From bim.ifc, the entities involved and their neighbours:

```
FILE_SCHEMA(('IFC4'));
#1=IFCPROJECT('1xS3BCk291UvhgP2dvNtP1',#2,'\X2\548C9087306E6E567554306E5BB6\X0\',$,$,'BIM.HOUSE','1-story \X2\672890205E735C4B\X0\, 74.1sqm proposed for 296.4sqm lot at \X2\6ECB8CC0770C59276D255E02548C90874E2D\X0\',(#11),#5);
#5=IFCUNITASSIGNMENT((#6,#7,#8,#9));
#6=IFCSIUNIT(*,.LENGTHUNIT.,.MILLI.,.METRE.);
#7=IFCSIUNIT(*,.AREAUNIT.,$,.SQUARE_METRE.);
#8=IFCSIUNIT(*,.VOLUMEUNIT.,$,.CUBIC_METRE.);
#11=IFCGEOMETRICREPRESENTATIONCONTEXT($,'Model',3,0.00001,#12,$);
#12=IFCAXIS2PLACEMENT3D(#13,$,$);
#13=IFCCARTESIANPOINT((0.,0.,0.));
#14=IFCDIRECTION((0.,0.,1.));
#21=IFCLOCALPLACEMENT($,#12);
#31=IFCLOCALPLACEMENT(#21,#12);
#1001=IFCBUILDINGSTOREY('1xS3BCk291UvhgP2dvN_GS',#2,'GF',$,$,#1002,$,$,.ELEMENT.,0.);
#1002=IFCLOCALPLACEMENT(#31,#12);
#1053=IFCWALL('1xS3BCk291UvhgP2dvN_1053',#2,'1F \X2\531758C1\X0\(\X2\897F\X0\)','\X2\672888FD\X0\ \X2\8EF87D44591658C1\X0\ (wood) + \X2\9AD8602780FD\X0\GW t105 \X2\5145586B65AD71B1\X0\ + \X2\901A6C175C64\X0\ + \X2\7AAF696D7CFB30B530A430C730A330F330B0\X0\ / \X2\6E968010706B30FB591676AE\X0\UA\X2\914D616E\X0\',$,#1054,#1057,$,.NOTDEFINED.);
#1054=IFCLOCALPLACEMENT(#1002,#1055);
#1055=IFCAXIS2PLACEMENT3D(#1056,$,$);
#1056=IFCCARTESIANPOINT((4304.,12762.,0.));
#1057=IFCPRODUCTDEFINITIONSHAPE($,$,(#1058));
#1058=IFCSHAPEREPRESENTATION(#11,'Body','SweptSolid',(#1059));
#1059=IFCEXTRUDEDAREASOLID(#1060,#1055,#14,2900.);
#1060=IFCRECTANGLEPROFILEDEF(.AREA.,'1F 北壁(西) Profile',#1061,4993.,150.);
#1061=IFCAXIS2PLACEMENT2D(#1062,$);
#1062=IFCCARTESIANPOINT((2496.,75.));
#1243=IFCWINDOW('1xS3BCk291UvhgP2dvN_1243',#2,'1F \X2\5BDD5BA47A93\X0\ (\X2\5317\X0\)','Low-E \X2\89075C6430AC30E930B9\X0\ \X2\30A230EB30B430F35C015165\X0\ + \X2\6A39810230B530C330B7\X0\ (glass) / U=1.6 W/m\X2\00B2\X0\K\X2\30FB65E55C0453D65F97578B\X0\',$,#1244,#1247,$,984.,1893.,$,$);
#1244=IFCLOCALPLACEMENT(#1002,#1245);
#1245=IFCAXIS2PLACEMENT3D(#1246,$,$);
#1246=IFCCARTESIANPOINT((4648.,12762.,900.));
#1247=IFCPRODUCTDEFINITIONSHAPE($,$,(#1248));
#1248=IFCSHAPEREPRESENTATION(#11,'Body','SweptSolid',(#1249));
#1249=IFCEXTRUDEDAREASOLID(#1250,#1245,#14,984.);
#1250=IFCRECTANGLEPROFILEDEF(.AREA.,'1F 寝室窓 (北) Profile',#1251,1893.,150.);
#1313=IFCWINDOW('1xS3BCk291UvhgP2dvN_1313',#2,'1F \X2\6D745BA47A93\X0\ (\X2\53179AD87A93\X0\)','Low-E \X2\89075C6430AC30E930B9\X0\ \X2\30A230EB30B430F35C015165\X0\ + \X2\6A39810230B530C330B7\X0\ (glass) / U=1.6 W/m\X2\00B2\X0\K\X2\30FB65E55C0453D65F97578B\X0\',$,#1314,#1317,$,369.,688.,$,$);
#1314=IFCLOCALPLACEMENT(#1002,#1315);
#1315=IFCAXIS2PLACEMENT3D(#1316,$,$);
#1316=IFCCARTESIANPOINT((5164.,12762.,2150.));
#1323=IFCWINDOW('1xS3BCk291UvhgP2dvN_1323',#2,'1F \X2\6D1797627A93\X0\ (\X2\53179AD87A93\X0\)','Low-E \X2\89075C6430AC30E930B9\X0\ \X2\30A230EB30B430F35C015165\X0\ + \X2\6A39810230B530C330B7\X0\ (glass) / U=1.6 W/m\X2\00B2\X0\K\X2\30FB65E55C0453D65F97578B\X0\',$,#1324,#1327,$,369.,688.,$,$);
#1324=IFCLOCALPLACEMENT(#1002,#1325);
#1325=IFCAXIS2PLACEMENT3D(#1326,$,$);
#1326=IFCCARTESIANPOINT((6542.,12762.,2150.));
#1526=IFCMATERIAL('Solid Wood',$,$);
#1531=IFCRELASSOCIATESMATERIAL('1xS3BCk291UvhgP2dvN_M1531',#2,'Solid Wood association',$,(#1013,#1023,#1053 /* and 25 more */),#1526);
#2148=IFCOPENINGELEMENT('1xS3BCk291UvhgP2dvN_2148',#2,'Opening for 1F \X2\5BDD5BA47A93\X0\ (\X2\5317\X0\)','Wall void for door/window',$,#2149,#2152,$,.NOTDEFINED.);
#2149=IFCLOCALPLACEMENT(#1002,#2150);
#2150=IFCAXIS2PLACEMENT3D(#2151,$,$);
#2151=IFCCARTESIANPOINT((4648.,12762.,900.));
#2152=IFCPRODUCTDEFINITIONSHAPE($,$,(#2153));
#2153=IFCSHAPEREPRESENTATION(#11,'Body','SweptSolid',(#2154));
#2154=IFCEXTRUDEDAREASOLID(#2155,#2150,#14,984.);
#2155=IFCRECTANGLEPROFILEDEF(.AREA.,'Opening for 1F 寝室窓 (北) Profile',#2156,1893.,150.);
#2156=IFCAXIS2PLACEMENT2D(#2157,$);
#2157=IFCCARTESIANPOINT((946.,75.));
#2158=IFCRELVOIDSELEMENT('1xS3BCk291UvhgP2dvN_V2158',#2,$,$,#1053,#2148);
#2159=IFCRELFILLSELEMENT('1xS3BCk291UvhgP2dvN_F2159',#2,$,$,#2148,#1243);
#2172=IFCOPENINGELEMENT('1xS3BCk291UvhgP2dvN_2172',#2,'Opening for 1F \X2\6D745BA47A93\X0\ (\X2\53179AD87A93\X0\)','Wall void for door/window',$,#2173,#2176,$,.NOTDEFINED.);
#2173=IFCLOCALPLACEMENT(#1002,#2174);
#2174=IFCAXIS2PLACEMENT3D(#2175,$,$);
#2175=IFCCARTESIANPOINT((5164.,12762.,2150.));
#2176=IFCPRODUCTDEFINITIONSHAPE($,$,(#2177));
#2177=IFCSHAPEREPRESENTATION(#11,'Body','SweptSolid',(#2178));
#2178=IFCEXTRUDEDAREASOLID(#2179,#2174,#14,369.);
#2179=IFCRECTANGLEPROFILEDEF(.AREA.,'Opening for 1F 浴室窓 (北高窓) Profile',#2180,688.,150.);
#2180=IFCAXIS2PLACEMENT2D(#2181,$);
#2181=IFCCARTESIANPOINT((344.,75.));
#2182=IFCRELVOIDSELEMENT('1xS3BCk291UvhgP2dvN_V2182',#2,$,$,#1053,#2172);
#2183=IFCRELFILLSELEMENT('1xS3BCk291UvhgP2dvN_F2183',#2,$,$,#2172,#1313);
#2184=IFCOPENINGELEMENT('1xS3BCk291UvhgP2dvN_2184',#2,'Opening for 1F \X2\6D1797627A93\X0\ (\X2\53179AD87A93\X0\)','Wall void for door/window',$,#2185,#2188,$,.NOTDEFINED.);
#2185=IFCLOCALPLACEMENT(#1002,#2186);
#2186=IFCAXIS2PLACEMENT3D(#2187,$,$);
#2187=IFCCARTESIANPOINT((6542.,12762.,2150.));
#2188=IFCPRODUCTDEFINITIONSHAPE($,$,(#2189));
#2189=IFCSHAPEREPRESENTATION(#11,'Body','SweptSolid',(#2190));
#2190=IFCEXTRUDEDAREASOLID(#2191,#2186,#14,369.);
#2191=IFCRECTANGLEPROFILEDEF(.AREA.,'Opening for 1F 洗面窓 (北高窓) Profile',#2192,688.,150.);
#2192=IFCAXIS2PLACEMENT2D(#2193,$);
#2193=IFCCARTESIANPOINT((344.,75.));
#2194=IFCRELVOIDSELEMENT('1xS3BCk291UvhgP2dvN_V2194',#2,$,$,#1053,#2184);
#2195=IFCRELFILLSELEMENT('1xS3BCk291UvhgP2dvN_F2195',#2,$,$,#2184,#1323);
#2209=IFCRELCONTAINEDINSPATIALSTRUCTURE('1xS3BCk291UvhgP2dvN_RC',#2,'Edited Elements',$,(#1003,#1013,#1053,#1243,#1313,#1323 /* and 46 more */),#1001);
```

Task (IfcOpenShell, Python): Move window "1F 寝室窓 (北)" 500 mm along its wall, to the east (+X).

```python
import ifcopenshell
import ifcopenshell.api.geometry
import ifcopenshell.util.placement
import ifcopenshell.util.unit

model = ifcopenshell.open("bim.ifc")
unit_scale = ifcopenshell.util.unit.calculate_unit_scale(model)

window = model.by_guid("1xS3BCk291UvhgP2dvN_1243")
opening = window.FillsVoids[0].RelatingOpeningElement
wall = opening.VoidsElements[0].RelatingBuildingElement

wall_matrix = ifcopenshell.util.placement.get_local_placement(wall.ObjectPlacement)
shift = wall_matrix[:3, 0] * 0.5 / unit_scale
before = ifcopenshell.util.placement.get_local_placement(window.ObjectPlacement)[:3, 3].copy()

# The window is not placed relative to its opening, so move both.
for product in (opening, window):
    matrix = ifcopenshell.util.placement.get_local_placement(product.ObjectPlacement)
    matrix[:3, 3] += shift
    ifcopenshell.api.geometry.edit_object_placement(model, product=product, matrix=matrix, is_si=False)

after = ifcopenshell.util.placement.get_local_placement(window.ObjectPlacement)[:3, 3]
print("window moved by", (after - before).round(3) + 0.0)

model.write("bim_updated.ifc")
```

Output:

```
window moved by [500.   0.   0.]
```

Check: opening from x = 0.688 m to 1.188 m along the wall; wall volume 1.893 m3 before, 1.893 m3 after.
